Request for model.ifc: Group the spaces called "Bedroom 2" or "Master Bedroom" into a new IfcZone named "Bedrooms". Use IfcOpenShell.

First a look at what the model holds.

```python
import ifcopenshell

model = ifcopenshell.open("model.ifc")
print(model.schema)
seen = {}
for space in model.by_type("IfcSpace"):
    seen[space.LongName] = seen.get(space.LongName, 0) + 1
for name, count in sorted(seen.items(), key=str):
    print(count, "x", name)
print("zones:", [z.Name for z in model.by_type("IfcZone")][:20])
```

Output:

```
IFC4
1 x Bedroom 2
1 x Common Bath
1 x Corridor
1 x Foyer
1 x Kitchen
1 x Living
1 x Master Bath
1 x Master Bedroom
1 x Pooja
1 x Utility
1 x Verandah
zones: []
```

```python
import ifcopenshell
import ifcopenshell.api.group
import ifcopenshell.api.root

model = ifcopenshell.open("model.ifc")

names = {"Bedroom 2", "Master Bedroom"}
spaces = [s for s in model.by_type("IfcSpace") if s.LongName in names]

zone = ifcopenshell.api.root.create_entity(model, ifc_class="IfcZone", name="Bedrooms")
ifcopenshell.api.group.assign_group(model, products=spaces, group=zone)
print(len(spaces), "spaces in", zone.Name)

model.write("model-out.ifc")
```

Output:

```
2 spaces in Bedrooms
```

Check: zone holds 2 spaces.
